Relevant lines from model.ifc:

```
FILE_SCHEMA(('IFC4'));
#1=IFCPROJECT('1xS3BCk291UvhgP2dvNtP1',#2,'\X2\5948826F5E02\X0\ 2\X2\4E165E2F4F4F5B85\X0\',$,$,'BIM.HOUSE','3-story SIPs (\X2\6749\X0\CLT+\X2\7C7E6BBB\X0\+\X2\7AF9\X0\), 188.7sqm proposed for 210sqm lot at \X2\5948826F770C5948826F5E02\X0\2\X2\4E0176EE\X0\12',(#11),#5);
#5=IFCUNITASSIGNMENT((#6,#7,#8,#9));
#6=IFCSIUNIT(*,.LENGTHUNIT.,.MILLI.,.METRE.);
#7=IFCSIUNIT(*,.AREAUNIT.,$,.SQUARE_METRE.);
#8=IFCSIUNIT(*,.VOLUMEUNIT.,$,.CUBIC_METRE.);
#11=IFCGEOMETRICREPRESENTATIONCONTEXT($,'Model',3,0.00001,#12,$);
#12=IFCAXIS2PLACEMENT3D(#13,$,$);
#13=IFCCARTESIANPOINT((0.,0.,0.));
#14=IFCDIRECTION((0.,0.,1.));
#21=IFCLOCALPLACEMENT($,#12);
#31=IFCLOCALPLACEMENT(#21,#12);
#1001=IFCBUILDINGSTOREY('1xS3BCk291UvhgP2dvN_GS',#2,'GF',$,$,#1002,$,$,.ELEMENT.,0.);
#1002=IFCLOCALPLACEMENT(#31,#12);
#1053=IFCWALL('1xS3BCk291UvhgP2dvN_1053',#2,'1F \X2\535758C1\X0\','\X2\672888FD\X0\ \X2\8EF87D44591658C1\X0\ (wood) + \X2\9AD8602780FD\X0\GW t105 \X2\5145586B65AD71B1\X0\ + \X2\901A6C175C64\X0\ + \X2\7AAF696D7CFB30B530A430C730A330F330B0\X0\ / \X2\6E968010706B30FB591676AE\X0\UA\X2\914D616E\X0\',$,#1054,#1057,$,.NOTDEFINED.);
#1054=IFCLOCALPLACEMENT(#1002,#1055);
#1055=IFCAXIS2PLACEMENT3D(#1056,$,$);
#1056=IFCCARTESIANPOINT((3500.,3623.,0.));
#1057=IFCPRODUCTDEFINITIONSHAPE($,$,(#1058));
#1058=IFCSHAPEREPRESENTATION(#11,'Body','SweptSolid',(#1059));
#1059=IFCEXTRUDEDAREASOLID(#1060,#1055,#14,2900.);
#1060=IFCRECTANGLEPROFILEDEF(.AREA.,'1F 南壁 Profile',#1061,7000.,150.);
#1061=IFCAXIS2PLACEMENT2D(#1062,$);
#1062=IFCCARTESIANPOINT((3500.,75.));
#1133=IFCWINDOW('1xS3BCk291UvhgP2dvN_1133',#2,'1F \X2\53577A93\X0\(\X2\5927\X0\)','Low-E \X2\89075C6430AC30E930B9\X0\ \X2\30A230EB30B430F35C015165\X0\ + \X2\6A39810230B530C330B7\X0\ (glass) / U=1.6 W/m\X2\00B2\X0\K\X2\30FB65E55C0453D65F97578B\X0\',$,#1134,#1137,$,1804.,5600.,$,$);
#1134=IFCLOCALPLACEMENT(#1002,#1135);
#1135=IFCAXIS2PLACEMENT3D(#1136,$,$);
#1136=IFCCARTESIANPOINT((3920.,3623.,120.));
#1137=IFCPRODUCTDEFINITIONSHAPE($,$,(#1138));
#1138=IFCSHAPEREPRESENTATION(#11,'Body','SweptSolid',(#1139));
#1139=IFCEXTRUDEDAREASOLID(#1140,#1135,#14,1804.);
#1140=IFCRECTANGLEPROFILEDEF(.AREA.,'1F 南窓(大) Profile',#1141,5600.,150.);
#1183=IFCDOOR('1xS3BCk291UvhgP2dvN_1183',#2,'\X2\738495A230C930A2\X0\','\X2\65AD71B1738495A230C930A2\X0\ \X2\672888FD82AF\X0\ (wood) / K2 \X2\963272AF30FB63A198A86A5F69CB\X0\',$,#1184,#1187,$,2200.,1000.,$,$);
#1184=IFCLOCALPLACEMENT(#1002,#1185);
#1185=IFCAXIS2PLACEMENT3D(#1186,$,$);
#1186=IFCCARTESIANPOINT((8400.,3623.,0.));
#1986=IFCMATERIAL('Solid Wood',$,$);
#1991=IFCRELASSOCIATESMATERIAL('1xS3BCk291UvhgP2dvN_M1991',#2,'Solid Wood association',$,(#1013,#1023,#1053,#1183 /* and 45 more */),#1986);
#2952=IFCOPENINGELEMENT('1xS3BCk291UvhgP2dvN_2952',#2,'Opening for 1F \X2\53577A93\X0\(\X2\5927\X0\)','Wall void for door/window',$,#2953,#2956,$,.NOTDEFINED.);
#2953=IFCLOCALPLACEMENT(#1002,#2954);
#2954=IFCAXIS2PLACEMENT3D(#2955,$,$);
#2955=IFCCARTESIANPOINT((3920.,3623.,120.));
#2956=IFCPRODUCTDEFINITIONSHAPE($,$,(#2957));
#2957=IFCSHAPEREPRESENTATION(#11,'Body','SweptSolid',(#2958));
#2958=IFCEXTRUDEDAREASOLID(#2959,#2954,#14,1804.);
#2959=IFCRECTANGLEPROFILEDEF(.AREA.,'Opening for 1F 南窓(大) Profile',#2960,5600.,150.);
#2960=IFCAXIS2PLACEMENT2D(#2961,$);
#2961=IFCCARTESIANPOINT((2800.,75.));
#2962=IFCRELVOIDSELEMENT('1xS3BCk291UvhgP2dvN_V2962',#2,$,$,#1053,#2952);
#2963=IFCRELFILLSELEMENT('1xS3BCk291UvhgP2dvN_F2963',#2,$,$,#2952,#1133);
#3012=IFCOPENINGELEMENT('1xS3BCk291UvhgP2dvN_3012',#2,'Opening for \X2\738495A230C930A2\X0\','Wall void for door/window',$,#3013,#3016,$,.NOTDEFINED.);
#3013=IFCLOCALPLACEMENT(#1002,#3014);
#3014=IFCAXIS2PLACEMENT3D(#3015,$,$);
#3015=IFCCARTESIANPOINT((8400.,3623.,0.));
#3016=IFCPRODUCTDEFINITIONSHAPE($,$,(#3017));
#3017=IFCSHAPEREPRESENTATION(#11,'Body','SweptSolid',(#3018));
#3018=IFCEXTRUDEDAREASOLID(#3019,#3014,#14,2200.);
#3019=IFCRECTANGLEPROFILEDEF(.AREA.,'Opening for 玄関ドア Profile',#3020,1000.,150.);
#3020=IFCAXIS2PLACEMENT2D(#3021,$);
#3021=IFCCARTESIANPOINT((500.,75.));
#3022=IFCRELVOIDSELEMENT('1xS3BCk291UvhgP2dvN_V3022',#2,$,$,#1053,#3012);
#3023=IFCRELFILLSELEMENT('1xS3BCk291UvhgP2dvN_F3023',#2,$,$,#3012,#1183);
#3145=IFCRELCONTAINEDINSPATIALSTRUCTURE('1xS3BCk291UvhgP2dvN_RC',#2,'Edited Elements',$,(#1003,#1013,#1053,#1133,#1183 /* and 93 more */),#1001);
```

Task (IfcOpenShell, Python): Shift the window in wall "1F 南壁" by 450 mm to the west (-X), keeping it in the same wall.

```python
import ifcopenshell
import ifcopenshell.api.geometry
import ifcopenshell.util.placement
import ifcopenshell.util.unit

model = ifcopenshell.open("model.ifc")
unit_scale = ifcopenshell.util.unit.calculate_unit_scale(model)

window = model.by_guid("1xS3BCk291UvhgP2dvN_1133")
opening = window.FillsVoids[0].RelatingOpeningElement
wall = opening.VoidsElements[0].RelatingBuildingElement

wall_matrix = ifcopenshell.util.placement.get_local_placement(wall.ObjectPlacement)
shift = wall_matrix[:3, 0] * -0.45 / unit_scale
before = ifcopenshell.util.placement.get_local_placement(window.ObjectPlacement)[:3, 3].copy()

# The window is not placed relative to its opening, so move both.
for product in (opening, window):
    matrix = ifcopenshell.util.placement.get_local_placement(product.ObjectPlacement)
    matrix[:3, 3] += shift
    ifcopenshell.api.geometry.edit_object_placement(model, product=product, matrix=matrix, is_si=False)

after = ifcopenshell.util.placement.get_local_placement(window.ObjectPlacement)[:3, 3]
print("window moved by", (after - before).round(3) + 0.0)

model.write("model-out.ifc")
```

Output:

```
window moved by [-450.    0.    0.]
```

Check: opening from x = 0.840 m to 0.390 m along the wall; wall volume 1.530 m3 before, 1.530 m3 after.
